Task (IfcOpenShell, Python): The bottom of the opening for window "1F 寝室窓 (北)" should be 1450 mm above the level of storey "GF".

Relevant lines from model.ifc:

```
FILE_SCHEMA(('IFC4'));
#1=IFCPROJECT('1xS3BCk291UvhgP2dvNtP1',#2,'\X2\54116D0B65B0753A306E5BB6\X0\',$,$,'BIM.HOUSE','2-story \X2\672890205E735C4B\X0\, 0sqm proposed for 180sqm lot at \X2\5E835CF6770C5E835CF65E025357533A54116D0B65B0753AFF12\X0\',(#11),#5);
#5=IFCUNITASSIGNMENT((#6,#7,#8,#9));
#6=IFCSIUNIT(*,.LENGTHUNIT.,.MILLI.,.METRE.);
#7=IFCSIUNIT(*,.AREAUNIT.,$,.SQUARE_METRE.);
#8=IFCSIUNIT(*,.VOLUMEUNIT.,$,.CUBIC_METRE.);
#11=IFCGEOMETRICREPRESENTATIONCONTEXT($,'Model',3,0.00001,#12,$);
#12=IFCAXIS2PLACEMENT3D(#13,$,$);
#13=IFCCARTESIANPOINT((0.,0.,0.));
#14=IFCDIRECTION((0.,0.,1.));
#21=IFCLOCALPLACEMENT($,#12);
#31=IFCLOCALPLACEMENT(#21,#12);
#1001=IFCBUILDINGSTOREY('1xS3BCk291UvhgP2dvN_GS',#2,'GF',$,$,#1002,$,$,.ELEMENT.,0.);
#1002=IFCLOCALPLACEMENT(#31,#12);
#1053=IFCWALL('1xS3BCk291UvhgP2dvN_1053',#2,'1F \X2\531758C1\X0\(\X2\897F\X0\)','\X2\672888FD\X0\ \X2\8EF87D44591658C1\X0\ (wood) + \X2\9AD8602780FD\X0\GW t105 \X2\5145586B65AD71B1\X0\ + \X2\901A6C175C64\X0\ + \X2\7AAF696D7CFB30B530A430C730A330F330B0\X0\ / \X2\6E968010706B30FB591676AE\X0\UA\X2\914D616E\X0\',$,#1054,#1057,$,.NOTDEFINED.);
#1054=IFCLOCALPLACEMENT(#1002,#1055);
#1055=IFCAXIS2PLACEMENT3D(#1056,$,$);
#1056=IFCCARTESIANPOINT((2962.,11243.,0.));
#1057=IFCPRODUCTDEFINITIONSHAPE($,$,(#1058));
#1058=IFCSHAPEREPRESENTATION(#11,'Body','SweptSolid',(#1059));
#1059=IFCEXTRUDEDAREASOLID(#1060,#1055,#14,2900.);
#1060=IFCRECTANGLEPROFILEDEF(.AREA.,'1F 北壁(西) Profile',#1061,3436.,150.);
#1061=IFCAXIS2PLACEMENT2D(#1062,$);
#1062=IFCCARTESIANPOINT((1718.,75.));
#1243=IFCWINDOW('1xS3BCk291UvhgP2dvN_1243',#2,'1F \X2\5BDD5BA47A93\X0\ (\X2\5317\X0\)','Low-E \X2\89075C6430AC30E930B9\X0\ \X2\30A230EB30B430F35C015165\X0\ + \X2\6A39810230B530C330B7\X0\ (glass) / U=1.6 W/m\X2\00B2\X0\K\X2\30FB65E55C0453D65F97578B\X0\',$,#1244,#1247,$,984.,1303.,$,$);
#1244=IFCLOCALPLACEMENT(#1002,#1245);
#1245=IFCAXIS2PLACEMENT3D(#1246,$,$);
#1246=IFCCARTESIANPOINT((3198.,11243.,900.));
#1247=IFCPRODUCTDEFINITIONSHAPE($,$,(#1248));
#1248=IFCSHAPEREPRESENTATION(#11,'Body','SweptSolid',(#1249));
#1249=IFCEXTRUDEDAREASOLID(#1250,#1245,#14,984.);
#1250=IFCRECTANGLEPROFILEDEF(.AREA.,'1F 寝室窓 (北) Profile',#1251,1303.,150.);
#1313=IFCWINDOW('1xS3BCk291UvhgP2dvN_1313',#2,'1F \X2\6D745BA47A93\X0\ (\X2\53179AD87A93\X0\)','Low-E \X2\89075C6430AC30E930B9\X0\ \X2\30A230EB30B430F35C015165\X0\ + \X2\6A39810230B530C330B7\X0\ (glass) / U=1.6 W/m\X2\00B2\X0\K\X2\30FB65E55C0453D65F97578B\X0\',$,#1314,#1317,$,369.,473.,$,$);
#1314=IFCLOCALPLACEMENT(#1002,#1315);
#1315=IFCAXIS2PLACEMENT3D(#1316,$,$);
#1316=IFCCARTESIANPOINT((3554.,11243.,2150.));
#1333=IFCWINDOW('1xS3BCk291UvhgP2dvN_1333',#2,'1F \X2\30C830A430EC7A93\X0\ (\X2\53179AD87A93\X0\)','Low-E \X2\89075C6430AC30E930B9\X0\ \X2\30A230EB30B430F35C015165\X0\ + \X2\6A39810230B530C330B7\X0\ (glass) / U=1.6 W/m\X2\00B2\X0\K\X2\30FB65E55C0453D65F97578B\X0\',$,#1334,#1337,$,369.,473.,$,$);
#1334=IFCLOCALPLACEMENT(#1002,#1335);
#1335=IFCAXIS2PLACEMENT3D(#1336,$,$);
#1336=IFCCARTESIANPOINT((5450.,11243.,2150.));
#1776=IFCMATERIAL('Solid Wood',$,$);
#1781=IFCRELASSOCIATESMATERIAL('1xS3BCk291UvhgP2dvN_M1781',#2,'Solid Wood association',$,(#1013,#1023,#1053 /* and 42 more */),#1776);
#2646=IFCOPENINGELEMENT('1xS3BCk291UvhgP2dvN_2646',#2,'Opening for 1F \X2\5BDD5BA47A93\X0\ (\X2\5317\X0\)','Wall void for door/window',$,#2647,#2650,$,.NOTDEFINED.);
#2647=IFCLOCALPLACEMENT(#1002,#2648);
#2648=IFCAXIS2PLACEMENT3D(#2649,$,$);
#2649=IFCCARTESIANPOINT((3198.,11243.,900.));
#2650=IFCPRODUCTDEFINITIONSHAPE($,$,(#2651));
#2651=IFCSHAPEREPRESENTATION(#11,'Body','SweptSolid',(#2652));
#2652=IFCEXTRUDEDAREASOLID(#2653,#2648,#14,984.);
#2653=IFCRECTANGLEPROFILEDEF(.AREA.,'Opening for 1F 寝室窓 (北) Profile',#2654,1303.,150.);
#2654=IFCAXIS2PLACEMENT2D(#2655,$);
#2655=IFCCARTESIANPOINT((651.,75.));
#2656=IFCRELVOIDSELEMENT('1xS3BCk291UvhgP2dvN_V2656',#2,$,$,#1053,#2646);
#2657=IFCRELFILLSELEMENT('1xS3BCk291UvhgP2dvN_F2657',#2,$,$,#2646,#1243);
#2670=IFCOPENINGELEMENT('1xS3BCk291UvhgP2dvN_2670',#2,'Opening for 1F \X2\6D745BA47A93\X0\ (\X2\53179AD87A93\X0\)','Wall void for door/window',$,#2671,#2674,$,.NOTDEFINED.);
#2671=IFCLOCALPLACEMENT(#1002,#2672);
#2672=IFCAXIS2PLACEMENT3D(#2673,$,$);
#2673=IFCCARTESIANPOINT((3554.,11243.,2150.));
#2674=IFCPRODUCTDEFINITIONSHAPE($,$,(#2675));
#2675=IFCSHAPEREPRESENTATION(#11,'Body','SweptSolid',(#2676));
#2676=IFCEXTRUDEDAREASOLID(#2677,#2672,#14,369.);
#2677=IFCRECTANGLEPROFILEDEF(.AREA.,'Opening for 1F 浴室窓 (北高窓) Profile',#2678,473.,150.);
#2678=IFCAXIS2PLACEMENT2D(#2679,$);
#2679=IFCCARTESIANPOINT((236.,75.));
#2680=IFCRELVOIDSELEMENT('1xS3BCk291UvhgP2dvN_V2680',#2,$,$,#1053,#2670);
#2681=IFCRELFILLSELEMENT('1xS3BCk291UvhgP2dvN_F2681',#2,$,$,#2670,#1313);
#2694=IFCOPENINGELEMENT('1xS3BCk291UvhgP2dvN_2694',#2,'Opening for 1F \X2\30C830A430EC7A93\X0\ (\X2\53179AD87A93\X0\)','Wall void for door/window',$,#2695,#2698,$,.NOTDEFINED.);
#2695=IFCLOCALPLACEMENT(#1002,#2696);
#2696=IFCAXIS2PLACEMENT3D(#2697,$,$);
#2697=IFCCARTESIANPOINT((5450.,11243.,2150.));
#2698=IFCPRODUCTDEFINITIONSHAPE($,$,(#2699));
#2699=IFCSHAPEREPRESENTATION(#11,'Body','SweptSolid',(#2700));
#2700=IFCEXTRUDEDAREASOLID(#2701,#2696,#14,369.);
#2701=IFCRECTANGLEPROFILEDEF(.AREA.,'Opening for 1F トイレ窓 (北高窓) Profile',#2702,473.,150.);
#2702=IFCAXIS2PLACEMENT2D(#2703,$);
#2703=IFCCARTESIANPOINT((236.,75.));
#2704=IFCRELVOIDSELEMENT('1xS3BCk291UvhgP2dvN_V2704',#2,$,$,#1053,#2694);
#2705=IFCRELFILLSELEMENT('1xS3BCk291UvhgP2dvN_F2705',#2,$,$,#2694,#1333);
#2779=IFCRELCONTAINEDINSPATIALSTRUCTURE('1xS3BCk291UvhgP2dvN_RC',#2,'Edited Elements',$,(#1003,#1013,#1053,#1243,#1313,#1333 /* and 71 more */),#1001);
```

```python
import numpy as np
import ifcopenshell
import ifcopenshell.api.geometry
import ifcopenshell.geom
import ifcopenshell.util.element
import ifcopenshell.util.placement
import ifcopenshell.util.shape
import ifcopenshell.util.unit

model = ifcopenshell.open("model.ifc")
unit_scale = ifcopenshell.util.unit.calculate_unit_scale(model)

window = model.by_guid("1xS3BCk291UvhgP2dvN_1243")
opening = window.FillsVoids[0].RelatingOpeningElement
storey = ifcopenshell.util.element.get_container(window, ifc_class="IfcBuildingStorey")
level = ifcopenshell.util.placement.get_local_placement(storey.ObjectPlacement)[2, 3]

# The opening's origin need not be at the sill, so measure its lowest point.
shape = ifcopenshell.geom.create_shape(ifcopenshell.geom.settings(), opening)
bottom = ifcopenshell.util.shape.get_shape_bottom_elevation(shape, shape.geometry) / unit_scale
dz = level + 1.45 / unit_scale - bottom

shift = np.array([0.0, 0.0, dz])
# The window is not placed relative to its opening, so move both.
for product in (opening, window):
    matrix = ifcopenshell.util.placement.get_local_placement(product.ObjectPlacement)
    matrix[:3, 3] += shift
    ifcopenshell.api.geometry.edit_object_placement(model, product=product, matrix=matrix, is_si=False)

print(f"moved by {dz * unit_scale:+.3f} m")

model.write("model-out.ifc")
```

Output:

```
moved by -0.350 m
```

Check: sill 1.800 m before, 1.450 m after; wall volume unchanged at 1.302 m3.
